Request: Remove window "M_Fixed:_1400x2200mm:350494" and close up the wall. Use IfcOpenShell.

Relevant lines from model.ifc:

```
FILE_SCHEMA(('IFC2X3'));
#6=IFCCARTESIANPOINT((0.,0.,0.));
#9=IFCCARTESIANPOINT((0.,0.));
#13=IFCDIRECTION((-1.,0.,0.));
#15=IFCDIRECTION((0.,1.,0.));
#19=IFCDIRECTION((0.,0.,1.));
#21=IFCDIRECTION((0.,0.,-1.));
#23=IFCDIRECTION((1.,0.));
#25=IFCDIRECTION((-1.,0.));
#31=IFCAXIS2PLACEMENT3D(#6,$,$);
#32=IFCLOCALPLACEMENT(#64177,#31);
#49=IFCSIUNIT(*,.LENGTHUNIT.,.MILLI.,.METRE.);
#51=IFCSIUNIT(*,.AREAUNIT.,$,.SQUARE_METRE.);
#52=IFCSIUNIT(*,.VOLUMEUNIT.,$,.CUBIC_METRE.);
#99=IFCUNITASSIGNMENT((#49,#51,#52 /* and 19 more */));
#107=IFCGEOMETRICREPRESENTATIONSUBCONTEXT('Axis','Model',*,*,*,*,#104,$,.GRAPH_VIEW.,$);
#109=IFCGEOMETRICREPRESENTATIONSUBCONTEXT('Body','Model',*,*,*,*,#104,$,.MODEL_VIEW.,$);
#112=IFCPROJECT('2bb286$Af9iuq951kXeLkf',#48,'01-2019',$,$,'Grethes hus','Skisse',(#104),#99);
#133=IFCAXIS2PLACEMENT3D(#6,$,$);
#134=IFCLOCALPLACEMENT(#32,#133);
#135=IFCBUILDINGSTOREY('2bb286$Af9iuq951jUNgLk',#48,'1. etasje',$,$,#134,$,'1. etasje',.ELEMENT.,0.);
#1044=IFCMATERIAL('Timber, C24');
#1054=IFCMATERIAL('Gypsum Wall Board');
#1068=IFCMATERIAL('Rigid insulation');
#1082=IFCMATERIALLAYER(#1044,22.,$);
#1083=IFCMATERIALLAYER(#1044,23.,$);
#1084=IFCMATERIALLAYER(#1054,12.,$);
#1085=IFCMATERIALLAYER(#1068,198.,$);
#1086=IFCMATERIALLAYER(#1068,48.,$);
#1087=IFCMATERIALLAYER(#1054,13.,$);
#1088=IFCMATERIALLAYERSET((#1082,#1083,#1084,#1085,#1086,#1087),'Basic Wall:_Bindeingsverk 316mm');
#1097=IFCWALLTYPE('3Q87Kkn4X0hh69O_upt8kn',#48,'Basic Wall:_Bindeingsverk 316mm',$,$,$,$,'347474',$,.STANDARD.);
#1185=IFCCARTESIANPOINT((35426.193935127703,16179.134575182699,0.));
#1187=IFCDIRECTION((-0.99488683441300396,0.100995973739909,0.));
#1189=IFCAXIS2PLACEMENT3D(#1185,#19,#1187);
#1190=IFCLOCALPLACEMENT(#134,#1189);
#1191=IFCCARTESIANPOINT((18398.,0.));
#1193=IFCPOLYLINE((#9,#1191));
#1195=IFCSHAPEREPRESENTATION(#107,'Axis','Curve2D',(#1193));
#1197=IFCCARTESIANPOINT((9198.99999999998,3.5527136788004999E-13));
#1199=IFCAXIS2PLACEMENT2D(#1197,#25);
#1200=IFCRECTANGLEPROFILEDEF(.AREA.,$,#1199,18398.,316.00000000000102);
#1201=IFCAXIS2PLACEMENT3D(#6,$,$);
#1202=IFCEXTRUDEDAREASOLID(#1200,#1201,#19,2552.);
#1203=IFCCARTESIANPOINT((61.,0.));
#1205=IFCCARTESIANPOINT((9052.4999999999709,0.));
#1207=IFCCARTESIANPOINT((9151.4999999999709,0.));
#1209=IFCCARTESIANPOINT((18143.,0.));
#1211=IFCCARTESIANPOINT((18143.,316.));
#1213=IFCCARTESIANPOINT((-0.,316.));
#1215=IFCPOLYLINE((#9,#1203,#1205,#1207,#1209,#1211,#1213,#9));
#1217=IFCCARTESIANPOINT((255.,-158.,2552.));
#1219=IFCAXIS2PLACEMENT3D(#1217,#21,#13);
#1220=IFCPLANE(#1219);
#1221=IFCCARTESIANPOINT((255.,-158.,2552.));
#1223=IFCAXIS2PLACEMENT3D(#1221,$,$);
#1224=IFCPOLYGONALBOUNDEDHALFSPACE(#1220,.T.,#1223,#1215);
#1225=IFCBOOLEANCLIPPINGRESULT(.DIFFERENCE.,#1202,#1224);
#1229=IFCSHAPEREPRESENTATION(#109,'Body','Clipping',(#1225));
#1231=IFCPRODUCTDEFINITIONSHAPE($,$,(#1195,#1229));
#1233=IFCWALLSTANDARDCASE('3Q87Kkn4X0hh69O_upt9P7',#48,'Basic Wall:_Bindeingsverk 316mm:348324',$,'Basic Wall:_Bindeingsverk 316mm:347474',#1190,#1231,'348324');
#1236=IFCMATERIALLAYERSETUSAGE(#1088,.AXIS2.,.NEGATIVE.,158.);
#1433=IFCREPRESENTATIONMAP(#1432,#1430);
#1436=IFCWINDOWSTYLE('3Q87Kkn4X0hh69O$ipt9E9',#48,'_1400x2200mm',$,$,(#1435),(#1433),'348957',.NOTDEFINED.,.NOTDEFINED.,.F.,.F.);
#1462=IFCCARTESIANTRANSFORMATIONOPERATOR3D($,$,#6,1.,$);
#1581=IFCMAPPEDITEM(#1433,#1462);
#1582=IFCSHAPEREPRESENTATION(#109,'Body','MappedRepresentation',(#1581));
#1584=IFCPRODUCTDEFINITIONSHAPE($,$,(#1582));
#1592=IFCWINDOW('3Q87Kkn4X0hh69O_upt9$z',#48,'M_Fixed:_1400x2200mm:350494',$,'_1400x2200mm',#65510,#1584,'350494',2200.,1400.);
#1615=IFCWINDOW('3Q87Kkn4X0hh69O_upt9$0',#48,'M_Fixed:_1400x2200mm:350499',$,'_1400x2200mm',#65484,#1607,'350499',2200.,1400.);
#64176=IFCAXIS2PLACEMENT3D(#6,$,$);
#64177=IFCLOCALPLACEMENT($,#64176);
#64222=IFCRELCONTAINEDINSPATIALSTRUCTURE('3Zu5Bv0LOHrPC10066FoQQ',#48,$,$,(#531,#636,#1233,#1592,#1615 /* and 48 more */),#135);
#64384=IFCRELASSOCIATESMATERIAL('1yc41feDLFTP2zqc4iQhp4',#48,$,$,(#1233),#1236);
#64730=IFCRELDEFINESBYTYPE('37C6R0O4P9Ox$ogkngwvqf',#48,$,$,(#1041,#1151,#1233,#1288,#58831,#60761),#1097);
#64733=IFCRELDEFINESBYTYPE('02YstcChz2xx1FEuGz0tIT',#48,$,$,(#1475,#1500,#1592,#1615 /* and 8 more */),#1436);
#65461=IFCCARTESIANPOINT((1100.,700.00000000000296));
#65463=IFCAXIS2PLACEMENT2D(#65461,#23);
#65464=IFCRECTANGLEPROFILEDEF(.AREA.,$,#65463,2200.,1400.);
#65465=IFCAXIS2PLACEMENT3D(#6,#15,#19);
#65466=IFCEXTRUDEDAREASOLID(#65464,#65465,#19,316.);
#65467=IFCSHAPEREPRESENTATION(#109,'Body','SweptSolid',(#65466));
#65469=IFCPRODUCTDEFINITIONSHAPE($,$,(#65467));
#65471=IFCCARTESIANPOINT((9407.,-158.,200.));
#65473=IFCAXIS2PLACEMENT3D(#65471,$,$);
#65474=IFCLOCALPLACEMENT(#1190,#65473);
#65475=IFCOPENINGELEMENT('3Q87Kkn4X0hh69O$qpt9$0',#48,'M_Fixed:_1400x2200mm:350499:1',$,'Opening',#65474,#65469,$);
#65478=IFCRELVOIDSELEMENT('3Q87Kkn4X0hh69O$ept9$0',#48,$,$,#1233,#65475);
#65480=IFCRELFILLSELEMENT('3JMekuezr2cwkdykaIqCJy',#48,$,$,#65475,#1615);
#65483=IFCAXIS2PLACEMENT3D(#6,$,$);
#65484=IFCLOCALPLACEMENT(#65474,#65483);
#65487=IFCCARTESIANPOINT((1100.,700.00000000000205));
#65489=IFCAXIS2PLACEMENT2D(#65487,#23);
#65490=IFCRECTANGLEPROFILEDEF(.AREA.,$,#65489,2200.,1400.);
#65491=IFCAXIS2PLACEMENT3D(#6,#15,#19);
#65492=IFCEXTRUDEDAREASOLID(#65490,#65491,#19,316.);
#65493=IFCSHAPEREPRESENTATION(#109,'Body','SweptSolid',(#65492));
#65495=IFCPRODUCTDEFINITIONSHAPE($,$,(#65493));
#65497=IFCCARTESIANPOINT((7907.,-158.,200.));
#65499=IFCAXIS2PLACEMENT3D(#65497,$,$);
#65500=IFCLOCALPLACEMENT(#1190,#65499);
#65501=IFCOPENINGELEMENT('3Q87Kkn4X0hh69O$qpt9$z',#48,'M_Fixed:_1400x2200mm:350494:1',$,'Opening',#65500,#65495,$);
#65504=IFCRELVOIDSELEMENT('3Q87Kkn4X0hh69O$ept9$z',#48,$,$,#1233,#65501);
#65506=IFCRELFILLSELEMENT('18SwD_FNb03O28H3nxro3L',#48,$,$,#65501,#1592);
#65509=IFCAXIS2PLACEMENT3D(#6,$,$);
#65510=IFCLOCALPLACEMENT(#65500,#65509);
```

```python
import ifcopenshell
import ifcopenshell.api.feature
import ifcopenshell.api.root
import ifcopenshell.geom
import ifcopenshell.util.shape

model = ifcopenshell.open("model.ifc")
settings = ifcopenshell.geom.settings()


def volume(element):
    """Net volume in cubic metres, openings subtracted."""
    shape = ifcopenshell.geom.create_shape(settings, element)
    return ifcopenshell.util.shape.get_volume(shape.geometry)


window = model.by_guid("3Q87Kkn4X0hh69O_upt9$z")
opening = window.FillsVoids[0].RelatingOpeningElement
wall = opening.VoidsElements[0].RelatingBuildingElement
before = volume(wall)

ifcopenshell.api.root.remove_product(model, product=window)
ifcopenshell.api.feature.remove_feature(model, feature=opening)

after = volume(wall)

print(f"wall volume {before:.3f} -> {after:.3f} m3")

model.write("model_edited.ifc")
```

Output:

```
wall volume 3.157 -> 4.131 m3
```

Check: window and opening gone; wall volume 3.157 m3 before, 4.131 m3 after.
